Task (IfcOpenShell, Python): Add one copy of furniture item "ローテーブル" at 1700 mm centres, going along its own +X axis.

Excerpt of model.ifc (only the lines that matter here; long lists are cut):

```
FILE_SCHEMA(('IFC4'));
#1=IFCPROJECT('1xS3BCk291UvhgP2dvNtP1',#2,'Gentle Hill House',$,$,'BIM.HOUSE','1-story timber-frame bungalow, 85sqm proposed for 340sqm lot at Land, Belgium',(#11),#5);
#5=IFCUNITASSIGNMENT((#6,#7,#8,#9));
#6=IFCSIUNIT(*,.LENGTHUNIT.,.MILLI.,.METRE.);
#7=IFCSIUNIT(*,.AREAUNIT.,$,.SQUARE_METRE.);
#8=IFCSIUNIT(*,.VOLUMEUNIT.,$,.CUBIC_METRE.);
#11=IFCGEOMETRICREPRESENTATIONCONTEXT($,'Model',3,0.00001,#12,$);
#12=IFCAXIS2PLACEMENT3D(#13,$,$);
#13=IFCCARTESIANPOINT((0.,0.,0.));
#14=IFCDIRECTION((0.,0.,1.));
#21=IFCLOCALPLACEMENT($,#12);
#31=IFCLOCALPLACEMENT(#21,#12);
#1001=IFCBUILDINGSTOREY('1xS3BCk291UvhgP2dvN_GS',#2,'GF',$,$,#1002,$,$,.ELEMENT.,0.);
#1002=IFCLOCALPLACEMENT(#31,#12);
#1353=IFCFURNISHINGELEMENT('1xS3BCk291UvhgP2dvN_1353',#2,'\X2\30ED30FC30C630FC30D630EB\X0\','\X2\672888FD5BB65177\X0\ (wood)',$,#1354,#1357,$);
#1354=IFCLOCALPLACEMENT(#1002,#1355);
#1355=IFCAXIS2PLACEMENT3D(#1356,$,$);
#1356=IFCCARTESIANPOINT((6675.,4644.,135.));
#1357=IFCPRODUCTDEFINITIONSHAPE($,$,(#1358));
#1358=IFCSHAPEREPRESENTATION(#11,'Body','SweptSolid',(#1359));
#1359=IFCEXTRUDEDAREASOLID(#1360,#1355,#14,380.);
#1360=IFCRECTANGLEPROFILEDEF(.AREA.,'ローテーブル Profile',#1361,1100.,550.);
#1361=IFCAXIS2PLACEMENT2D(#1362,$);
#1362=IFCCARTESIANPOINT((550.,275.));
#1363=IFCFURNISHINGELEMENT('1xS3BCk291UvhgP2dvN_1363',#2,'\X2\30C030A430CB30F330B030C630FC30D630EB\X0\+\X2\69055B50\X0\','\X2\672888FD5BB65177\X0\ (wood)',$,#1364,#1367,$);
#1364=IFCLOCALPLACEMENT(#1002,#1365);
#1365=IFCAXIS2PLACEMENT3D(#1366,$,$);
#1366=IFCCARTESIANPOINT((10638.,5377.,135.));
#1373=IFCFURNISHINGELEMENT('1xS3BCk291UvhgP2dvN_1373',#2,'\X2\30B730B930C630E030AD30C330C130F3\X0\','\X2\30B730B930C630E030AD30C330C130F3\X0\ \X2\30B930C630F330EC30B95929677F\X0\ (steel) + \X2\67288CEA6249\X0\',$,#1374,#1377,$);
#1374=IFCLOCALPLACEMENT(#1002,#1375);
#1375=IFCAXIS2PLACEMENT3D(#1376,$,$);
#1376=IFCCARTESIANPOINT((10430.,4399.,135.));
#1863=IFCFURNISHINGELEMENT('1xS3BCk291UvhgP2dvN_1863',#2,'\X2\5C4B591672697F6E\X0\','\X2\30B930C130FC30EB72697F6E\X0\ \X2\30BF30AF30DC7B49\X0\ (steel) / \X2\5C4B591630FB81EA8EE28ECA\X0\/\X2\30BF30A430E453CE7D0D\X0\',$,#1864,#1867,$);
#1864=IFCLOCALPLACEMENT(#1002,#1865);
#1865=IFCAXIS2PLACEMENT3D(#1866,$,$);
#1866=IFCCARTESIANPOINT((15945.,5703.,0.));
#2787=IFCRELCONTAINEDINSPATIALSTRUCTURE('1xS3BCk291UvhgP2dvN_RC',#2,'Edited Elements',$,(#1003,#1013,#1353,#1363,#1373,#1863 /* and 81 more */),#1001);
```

```python
import ifcopenshell
import ifcopenshell.api.geometry
import ifcopenshell.api.root
import ifcopenshell.util.element
import ifcopenshell.util.placement

model = ifcopenshell.open("model.ifc")


def reuse_history(source, copy):
    """copy_class also copies each property set's owner history, people and application; keep the originals."""
    for rel in copy.IsDefinedBy:
        if rel.is_a("IfcRelDefinesByProperties") and (history := rel.RelatingPropertyDefinition.OwnerHistory):
            rel.RelatingPropertyDefinition.OwnerHistory = source.OwnerHistory
            ifcopenshell.util.element.remove_deep2(model, history)


source = model.by_id(1353)
base = ifcopenshell.util.placement.get_local_placement(source.ObjectPlacement)
step = base[:3, 0] * 1700.0

for i in range(1, 2):
    copy = ifcopenshell.api.root.copy_class(model, product=source)
    copy.Representation = ifcopenshell.util.element.copy_deep(
        model, source.Representation, exclude=["IfcGeometricRepresentationContext", "IfcRepresentationMap"]
    )
    reuse_history(source, copy)
    matrix = base.copy()
    matrix[:3, 3] += i * step
    print("added at", matrix[:3, 3].round(3) + 0.0)
    ifcopenshell.api.geometry.edit_object_placement(model, product=copy, matrix=matrix, is_si=False)

model.write("model_edited.ifc")
```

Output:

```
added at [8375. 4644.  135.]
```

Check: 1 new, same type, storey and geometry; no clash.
